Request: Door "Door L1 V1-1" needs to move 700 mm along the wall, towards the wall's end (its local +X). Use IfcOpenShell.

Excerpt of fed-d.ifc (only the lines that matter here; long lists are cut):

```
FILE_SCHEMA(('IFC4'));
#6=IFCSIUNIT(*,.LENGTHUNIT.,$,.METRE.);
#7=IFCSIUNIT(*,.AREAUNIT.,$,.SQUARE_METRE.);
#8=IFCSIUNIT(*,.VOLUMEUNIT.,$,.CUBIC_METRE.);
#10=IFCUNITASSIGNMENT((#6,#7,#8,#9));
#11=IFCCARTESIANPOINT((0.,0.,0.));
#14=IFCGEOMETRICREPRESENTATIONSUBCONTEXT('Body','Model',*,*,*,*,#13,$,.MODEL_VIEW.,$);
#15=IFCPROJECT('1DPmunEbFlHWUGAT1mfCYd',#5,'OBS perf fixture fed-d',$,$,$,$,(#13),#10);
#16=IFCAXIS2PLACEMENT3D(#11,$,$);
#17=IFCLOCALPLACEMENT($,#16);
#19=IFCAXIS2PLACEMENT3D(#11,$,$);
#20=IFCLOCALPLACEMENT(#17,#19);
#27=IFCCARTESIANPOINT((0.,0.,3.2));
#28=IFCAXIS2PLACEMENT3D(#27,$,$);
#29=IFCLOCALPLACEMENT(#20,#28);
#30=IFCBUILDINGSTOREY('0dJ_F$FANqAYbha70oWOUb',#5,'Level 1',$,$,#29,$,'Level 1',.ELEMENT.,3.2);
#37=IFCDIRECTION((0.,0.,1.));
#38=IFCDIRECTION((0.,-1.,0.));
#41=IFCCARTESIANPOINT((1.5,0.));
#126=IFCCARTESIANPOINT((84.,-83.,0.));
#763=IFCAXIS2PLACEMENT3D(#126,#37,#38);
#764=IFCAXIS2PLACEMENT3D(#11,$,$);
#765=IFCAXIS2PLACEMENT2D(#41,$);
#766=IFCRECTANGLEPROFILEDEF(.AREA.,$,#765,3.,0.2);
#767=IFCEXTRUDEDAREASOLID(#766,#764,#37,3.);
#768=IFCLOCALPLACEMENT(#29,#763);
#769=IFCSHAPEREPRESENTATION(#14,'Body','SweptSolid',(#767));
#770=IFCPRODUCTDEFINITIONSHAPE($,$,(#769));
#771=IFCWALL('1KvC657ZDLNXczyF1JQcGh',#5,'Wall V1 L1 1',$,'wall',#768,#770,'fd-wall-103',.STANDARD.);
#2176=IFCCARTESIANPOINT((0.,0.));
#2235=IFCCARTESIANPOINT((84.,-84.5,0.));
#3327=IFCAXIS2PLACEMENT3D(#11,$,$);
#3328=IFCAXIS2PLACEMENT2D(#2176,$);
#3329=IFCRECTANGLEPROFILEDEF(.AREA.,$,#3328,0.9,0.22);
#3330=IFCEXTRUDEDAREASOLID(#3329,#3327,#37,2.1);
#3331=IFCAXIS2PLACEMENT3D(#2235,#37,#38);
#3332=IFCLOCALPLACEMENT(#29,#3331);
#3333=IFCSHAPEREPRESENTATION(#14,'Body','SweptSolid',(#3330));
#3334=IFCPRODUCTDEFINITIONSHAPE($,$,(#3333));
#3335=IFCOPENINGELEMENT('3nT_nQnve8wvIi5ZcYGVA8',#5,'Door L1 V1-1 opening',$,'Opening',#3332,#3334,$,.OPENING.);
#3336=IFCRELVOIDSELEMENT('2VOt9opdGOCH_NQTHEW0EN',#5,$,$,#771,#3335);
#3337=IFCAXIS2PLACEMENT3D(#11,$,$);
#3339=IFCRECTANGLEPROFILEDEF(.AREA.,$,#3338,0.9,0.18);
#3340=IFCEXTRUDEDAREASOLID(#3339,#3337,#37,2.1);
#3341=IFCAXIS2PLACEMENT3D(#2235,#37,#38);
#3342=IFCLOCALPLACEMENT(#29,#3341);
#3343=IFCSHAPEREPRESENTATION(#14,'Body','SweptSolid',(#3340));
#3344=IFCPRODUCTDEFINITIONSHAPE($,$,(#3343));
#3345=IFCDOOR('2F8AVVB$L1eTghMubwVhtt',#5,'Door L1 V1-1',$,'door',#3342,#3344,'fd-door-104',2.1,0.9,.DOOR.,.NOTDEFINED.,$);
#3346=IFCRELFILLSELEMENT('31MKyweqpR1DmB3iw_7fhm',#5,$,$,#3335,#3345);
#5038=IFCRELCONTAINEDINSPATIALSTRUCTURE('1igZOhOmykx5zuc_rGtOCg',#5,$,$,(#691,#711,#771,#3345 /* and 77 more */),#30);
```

```python
import ifcopenshell
import ifcopenshell.api.geometry
import ifcopenshell.util.placement
import ifcopenshell.util.unit

model = ifcopenshell.open("fed-d.ifc")
unit_scale = ifcopenshell.util.unit.calculate_unit_scale(model)

door = model.by_guid("2F8AVVB$L1eTghMubwVhtt")
opening = door.FillsVoids[0].RelatingOpeningElement
wall = opening.VoidsElements[0].RelatingBuildingElement

wall_matrix = ifcopenshell.util.placement.get_local_placement(wall.ObjectPlacement)
shift = wall_matrix[:3, 0] * 0.7 / unit_scale
before = ifcopenshell.util.placement.get_local_placement(door.ObjectPlacement)[:3, 3].copy()

# The door is not placed relative to its opening, so move both.
for product in (opening, door):
    matrix = ifcopenshell.util.placement.get_local_placement(product.ObjectPlacement)
    matrix[:3, 3] += shift
    ifcopenshell.api.geometry.edit_object_placement(model, product=product, matrix=matrix, is_si=False)

after = ifcopenshell.util.placement.get_local_placement(door.ObjectPlacement)[:3, 3]
print("door moved by", (after - before).round(3) + 0.0)

model.write("fed-d-out.ifc")
```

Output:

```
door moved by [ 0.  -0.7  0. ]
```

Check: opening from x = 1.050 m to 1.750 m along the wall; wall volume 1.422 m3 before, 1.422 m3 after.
